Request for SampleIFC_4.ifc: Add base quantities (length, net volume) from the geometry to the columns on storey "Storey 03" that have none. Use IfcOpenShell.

First a look at what the model holds.

```python
import ifcopenshell
import ifcopenshell.util.element
import ifcopenshell.util.unit

model = ifcopenshell.open("SampleIFC_4.ifc")
print(model.schema)
for unit_type in ("LENGTHUNIT", "AREAUNIT", "VOLUMEUNIT"):
    print(unit_type, ifcopenshell.util.unit.calculate_unit_scale(model, unit_type))
storey = next(s for s in model.by_type("IfcBuildingStorey") if s.Name == "Storey 03")
columns = [e for e in ifcopenshell.util.element.get_decomposition(storey) if e.is_a("IfcColumn")]
for e in sorted(columns, key=lambda e: e.id()):
    print(e.id(), e.is_a(), e.Name, list(ifcopenshell.util.element.get_psets(e, qtos_only=True)), sep=" | ")
```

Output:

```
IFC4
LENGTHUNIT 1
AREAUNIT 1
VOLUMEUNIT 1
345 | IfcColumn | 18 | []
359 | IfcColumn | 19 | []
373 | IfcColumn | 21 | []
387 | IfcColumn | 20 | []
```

```python
import ifcopenshell
import ifcopenshell.api.pset
import ifcopenshell.geom
import ifcopenshell.util.element
import ifcopenshell.util.shape
import ifcopenshell.util.unit

model = ifcopenshell.open("SampleIFC_4.ifc")
unit_scale = ifcopenshell.util.unit.calculate_unit_scale(model)
volume_scale = ifcopenshell.util.unit.calculate_unit_scale(model, "VOLUMEUNIT")
settings = ifcopenshell.geom.settings()

storey = next(s for s in model.by_type("IfcBuildingStorey") if s.Name == "Storey 03")
columns = [e for e in ifcopenshell.util.element.get_decomposition(storey) if e.is_a("IfcColumn")]

for e in sorted(columns, key=lambda e: e.id()):
    if ifcopenshell.util.element.get_psets(e, qtos_only=True, should_inherit=False):
        continue
    # Geometry comes back in metres, in the element's own axes.
    shape = ifcopenshell.geom.create_shape(settings, e)
    values = {
        "Length": ifcopenshell.util.shape.get_z(shape.geometry) / unit_scale,
        "NetVolume": ifcopenshell.util.shape.get_volume(shape.geometry) / volume_scale,
    }
    qto = ifcopenshell.api.pset.add_qto(model, product=e, name="Qto_ColumnBaseQuantities")
    ifcopenshell.api.pset.edit_qto(model, qto=qto, properties=values)
    print(e.id(), {k: round(v, 3) for k, v in values.items()})

model.write("SampleIFC_4-out.ifc")
```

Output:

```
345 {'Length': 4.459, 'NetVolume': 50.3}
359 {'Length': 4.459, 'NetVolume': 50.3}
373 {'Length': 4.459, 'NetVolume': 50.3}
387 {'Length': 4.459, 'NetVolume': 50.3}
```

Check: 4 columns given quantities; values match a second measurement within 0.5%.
